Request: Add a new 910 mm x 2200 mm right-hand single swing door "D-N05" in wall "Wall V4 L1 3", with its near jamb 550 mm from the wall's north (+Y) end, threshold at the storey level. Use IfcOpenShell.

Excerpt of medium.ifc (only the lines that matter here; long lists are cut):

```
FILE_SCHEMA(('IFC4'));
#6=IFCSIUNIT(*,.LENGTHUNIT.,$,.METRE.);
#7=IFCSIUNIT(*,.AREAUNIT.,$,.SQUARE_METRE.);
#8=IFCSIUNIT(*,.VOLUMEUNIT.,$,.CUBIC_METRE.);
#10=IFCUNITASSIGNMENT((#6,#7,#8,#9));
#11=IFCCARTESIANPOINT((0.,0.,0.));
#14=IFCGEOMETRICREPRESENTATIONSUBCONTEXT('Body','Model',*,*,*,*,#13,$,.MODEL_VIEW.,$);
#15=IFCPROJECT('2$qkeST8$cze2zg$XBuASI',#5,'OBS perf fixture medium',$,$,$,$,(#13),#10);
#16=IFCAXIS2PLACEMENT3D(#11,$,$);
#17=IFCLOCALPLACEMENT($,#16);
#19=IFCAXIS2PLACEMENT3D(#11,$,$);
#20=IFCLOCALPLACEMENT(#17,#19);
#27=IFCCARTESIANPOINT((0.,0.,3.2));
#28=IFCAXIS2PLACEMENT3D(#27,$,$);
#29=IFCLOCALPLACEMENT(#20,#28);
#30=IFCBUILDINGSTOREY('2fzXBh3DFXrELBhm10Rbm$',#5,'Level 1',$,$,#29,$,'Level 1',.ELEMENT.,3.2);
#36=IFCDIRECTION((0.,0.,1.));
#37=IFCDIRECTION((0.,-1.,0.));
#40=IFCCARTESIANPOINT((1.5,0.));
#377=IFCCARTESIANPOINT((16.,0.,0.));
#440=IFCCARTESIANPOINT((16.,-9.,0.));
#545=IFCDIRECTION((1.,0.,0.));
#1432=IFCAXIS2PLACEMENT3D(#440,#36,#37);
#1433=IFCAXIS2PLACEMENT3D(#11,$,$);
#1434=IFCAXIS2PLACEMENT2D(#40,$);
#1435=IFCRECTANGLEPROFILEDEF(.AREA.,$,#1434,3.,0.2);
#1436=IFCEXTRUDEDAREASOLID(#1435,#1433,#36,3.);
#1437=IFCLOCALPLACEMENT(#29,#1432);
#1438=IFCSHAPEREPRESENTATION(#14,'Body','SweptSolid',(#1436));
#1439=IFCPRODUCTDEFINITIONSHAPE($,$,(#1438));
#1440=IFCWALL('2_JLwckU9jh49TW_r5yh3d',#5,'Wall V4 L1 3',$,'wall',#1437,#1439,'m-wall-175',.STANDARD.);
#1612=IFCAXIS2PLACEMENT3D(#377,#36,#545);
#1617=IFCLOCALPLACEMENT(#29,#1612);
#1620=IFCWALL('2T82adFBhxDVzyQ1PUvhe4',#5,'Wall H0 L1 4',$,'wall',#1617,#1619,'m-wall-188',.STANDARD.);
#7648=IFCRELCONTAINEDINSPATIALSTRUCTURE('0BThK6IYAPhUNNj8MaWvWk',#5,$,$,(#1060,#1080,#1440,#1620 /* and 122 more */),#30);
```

```python
import numpy as np
import ifcopenshell
import ifcopenshell.api.feature
import ifcopenshell.api.geometry
import ifcopenshell.api.root
import ifcopenshell.api.spatial
import ifcopenshell.geom
import ifcopenshell.util.element
import ifcopenshell.util.placement
import ifcopenshell.util.representation
import ifcopenshell.util.shape
import ifcopenshell.util.unit

model = ifcopenshell.open("medium.ifc")
unit_scale = ifcopenshell.util.unit.calculate_unit_scale(model)
settings = ifcopenshell.geom.settings()


def volume(element):
    """Net volume in cubic metres, openings subtracted."""
    shape = ifcopenshell.geom.create_shape(settings, element)
    return ifcopenshell.util.shape.get_volume(shape.geometry)


wall = model.by_guid("2_JLwckU9jh49TW_r5yh3d")
storey = ifcopenshell.util.element.get_container(wall, ifc_class="IfcBuildingStorey")
context = ifcopenshell.util.representation.get_context(model, "Model", "Body", "MODEL_VIEW")
before = volume(wall)

width, height, from_end, sill = 0.91, 2.2, 0.55, 0.0  # metres

# The wall runs along its own X axis, and the end named is its -X end.
wall_shape = ifcopenshell.geom.create_shape(settings, wall)
x, y, z = ifcopenshell.util.shape.get_vertices(wall_shape.geometry).T
start = x.min() + from_end
face, thickness = float(y.min()), float(y.max() - y.min())
wall_matrix = ifcopenshell.util.placement.get_local_placement(wall.ObjectPlacement)
level = ifcopenshell.util.placement.get_local_placement(storey.ObjectPlacement)[2, 3]


def in_wall(x, y):
    """Placement at x, y metres in the wall's axes, at sill height."""
    matrix = wall_matrix.copy()
    matrix[:, 3] = wall_matrix @ np.array([x / unit_scale, y / unit_scale, 0.0, 1.0])
    matrix[2, 3] = level + sill / unit_scale
    return matrix


# Opening: a box that overshoots both wall faces by 50 mm.
opening = ifcopenshell.api.root.create_entity(model, ifc_class="IfcOpeningElement", predefined_type="OPENING")
box = ifcopenshell.api.geometry.add_wall_representation(
    model, context=context, length=width, height=height, thickness=thickness + 0.1
)
ifcopenshell.api.geometry.assign_representation(model, product=opening, representation=box)
ifcopenshell.api.geometry.edit_object_placement(model, product=opening, matrix=in_wall(start, face - 0.05), is_si=False)
ifcopenshell.api.feature.add_feature(model, feature=opening, element=wall)

door = ifcopenshell.api.root.create_entity(model, ifc_class="IfcDoor", name="D-N05", predefined_type="DOOR")
door.OverallWidth, door.OverallHeight = width / unit_scale, height / unit_scale
door.OperationType = "SINGLE_SWING_RIGHT"
body = ifcopenshell.api.geometry.add_door_representation(
    model,
    context=context,
    overall_width=door.OverallWidth,
    overall_height=door.OverallHeight,
    operation_type="SINGLE_SWING_RIGHT",
    lining_properties={"LiningDepth": thickness / unit_scale, "ThresholdDepth": thickness / unit_scale},
)
ifcopenshell.api.geometry.assign_representation(model, product=door, representation=body)
ifcopenshell.api.spatial.assign_container(model, products=[door], relating_structure=storey)
ifcopenshell.api.feature.add_filling(model, opening=opening, element=door)

# The lining spans the wall, so the door starts at the wall face.
ifcopenshell.api.geometry.edit_object_placement(model, product=door, matrix=in_wall(start, face), is_si=False)

after = volume(wall)

print(f"wall volume {before:.3f} -> {after:.3f} m3")

model.write("medium_edited.ifc")
```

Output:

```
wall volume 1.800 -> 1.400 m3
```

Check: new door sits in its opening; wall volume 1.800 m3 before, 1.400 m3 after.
